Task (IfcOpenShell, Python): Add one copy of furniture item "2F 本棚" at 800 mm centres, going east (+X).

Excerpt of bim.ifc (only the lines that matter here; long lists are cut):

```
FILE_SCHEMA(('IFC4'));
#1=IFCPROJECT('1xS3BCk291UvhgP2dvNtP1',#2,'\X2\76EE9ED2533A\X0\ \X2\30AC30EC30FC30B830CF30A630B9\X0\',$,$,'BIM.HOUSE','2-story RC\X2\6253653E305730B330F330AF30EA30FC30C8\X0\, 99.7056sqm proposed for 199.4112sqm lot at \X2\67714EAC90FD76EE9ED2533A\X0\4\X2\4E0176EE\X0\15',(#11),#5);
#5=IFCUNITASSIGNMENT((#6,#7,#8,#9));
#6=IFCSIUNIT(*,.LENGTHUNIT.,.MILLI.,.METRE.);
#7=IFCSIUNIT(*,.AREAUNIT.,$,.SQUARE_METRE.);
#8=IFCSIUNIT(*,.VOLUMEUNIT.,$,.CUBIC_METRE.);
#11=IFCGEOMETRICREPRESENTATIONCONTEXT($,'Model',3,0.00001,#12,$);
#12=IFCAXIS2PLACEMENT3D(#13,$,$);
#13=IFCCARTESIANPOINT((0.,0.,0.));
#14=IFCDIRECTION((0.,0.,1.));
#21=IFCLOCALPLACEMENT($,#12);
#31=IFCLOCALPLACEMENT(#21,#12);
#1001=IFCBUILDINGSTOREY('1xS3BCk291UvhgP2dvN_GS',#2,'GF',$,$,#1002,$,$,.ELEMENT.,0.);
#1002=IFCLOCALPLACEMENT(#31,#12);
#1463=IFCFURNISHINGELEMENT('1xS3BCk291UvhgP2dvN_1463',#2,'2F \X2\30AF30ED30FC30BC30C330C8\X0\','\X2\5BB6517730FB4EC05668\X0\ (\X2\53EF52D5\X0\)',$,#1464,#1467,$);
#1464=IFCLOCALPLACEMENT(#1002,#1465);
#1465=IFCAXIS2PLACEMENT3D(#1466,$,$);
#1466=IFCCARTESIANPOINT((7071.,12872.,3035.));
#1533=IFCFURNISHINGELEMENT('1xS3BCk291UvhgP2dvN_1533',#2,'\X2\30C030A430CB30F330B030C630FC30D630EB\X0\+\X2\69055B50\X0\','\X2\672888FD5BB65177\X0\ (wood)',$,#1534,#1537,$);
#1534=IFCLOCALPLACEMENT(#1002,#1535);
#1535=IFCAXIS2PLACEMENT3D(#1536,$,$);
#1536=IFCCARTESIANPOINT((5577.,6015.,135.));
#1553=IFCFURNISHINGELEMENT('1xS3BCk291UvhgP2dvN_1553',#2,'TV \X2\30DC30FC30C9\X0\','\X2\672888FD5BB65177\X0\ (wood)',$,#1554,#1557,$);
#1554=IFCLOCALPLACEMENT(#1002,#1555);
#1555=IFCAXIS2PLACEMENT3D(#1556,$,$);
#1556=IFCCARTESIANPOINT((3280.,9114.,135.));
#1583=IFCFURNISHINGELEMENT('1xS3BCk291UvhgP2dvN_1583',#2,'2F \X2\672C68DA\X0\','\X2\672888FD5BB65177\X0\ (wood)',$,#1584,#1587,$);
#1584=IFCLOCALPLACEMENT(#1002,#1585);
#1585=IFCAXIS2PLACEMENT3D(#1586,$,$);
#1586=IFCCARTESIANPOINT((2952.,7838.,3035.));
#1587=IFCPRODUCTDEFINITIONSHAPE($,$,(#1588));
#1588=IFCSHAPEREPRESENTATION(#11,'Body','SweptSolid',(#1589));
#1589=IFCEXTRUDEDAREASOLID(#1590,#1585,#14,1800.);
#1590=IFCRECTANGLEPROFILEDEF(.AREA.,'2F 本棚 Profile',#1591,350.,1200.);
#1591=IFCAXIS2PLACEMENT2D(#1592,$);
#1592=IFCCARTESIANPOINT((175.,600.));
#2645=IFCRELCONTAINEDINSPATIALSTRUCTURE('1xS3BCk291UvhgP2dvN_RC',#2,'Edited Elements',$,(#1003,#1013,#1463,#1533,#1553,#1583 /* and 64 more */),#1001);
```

```python
import numpy as np
import ifcopenshell
import ifcopenshell.api.geometry
import ifcopenshell.api.root
import ifcopenshell.util.element
import ifcopenshell.util.placement

model = ifcopenshell.open("bim.ifc")


def reuse_history(source, copy):
    """copy_class also copies each property set's owner history, people and application; keep the originals."""
    for rel in copy.IsDefinedBy:
        if rel.is_a("IfcRelDefinesByProperties") and (history := rel.RelatingPropertyDefinition.OwnerHistory):
            rel.RelatingPropertyDefinition.OwnerHistory = source.OwnerHistory
            ifcopenshell.util.element.remove_deep2(model, history)


source = model.by_id(1583)
base = ifcopenshell.util.placement.get_local_placement(source.ObjectPlacement)
step = np.array([1.0, 0.0, 0.0]) * 800.0

for i in range(1, 2):
    copy = ifcopenshell.api.root.copy_class(model, product=source)
    copy.Representation = ifcopenshell.util.element.copy_deep(
        model, source.Representation, exclude=["IfcGeometricRepresentationContext", "IfcRepresentationMap"]
    )
    reuse_history(source, copy)
    matrix = base.copy()
    matrix[:3, 3] += i * step
    print("added at", matrix[:3, 3].round(3) + 0.0)
    ifcopenshell.api.geometry.edit_object_placement(model, product=copy, matrix=matrix, is_si=False)

model.write("bim_updated.ifc")
```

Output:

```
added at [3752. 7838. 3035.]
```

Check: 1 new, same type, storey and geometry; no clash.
